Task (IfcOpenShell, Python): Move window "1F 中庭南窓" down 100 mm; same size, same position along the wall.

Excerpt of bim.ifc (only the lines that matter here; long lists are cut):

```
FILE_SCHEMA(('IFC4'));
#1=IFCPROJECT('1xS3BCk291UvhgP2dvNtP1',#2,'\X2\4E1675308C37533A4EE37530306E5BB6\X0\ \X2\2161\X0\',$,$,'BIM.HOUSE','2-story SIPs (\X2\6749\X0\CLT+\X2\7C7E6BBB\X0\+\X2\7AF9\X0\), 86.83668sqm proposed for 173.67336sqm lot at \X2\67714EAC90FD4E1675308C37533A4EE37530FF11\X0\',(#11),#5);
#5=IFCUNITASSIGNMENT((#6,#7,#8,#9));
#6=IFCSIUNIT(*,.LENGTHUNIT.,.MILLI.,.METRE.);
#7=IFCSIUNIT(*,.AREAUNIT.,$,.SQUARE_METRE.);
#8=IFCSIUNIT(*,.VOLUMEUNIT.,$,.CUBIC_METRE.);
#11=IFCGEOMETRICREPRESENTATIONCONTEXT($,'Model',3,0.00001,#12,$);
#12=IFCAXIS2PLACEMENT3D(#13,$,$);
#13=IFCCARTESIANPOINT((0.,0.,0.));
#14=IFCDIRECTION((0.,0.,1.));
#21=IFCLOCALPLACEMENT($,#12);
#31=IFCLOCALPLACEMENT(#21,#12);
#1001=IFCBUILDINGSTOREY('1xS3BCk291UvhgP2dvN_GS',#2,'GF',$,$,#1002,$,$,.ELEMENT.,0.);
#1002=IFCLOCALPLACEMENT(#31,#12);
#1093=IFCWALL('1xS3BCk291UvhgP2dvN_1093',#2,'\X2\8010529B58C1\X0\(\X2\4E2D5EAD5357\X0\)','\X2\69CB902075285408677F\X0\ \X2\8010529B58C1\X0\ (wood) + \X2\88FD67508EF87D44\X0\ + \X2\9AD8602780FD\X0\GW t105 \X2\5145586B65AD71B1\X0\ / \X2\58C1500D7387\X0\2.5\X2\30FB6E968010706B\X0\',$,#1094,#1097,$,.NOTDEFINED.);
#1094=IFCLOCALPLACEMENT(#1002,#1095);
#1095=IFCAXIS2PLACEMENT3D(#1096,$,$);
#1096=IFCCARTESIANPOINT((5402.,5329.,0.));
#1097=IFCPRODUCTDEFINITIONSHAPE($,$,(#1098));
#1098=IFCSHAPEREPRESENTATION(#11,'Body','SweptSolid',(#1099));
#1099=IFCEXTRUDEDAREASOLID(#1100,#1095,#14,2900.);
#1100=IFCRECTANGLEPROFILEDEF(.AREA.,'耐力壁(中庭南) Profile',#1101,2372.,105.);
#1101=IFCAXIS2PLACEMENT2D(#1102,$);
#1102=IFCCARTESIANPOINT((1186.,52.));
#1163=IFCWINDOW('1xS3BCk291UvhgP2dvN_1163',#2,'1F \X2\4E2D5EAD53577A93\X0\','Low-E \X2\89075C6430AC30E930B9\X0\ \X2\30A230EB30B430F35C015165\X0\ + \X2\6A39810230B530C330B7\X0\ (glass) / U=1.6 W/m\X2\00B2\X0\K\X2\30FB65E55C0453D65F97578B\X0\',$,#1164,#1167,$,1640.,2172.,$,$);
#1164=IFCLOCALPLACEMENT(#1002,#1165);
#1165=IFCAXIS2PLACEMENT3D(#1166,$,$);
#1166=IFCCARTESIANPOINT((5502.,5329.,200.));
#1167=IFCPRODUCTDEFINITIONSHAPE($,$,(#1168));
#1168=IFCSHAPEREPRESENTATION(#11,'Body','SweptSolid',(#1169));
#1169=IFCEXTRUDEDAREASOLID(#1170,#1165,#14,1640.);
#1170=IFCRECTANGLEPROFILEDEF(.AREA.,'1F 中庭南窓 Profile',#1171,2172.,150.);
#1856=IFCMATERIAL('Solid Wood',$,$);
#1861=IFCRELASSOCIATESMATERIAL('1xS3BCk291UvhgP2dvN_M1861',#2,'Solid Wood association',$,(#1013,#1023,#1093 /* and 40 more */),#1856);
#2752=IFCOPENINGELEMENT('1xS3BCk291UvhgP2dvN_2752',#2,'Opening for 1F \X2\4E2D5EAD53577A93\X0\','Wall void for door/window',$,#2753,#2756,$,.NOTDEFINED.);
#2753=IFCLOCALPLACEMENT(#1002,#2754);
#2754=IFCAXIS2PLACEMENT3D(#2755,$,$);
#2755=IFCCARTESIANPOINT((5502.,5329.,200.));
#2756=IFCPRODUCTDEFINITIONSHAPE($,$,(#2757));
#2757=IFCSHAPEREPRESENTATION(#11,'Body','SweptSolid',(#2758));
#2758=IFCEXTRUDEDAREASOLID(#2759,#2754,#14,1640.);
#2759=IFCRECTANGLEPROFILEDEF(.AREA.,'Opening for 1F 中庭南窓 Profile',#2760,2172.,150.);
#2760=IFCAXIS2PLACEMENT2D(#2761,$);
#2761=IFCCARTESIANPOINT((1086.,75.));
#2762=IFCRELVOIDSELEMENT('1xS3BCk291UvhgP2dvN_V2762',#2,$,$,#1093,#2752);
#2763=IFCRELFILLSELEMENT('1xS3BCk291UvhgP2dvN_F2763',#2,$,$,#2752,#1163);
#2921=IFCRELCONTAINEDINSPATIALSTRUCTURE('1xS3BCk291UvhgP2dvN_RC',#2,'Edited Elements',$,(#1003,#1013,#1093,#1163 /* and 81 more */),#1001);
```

```python
import numpy as np
import ifcopenshell
import ifcopenshell.api.geometry
import ifcopenshell.util.placement
import ifcopenshell.util.unit

model = ifcopenshell.open("bim.ifc")
unit_scale = ifcopenshell.util.unit.calculate_unit_scale(model)

window = model.by_guid("1xS3BCk291UvhgP2dvN_1163")
opening = window.FillsVoids[0].RelatingOpeningElement
dz = -100.0

shift = np.array([0.0, 0.0, dz])
# The window is not placed relative to its opening, so move both.
for product in (opening, window):
    matrix = ifcopenshell.util.placement.get_local_placement(product.ObjectPlacement)
    matrix[:3, 3] += shift
    ifcopenshell.api.geometry.edit_object_placement(model, product=product, matrix=matrix, is_si=False)

print(f"moved by {dz * unit_scale:+.3f} m")

model.write("bim_updated.ifc")
```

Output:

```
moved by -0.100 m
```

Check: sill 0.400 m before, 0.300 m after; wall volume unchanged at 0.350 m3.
